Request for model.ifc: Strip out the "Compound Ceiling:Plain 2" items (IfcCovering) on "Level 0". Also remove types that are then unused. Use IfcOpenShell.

First a look at what the model holds.

```python
import ifcopenshell
import ifcopenshell.util.element

model = ifcopenshell.open("model.ifc")
print(model.schema)
storey = next(s for s in model.by_type("IfcBuildingStorey") if s.Name == "Level 0")
coverings = [e for e in ifcopenshell.util.element.get_decomposition(storey) if e.is_a("IfcCovering")]
seen = {}
for e in coverings:
    element_type = ifcopenshell.util.element.get_type(e)
    name = element_type.Name if element_type not in (None, e) else None
    seen[name] = seen.get(name, 0) + 1
for name, count in sorted(seen.items(), key=str):
    print(count, "x", name)
```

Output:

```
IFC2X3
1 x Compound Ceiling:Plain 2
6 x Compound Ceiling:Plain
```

```python
import ifcopenshell
import ifcopenshell.api.root
import ifcopenshell.util.element

model = ifcopenshell.open("model.ifc")

storey = next(s for s in model.by_type("IfcBuildingStorey") if s.Name == "Level 0")
coverings = [e for e in ifcopenshell.util.element.get_decomposition(storey) if e.is_a("IfcCovering")]
targets = [e for e in coverings if (t := ifcopenshell.util.element.get_type(e)) not in (None, e) and t.Name == "Compound Ceiling:Plain 2"]
types = {ifcopenshell.util.element.get_type(e) for e in targets} - {None, *targets}

for e in targets:
    ifcopenshell.api.root.remove_product(model, product=e)
print(len(targets), "removed")

unused = [t for t in types if not ifcopenshell.util.element.get_types(t)]
for t in unused:
    ifcopenshell.api.root.remove_product(model, product=t)
print(len(unused), "unused types removed")

model.write("model_rev.ifc")
```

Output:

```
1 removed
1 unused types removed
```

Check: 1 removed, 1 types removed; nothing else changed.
